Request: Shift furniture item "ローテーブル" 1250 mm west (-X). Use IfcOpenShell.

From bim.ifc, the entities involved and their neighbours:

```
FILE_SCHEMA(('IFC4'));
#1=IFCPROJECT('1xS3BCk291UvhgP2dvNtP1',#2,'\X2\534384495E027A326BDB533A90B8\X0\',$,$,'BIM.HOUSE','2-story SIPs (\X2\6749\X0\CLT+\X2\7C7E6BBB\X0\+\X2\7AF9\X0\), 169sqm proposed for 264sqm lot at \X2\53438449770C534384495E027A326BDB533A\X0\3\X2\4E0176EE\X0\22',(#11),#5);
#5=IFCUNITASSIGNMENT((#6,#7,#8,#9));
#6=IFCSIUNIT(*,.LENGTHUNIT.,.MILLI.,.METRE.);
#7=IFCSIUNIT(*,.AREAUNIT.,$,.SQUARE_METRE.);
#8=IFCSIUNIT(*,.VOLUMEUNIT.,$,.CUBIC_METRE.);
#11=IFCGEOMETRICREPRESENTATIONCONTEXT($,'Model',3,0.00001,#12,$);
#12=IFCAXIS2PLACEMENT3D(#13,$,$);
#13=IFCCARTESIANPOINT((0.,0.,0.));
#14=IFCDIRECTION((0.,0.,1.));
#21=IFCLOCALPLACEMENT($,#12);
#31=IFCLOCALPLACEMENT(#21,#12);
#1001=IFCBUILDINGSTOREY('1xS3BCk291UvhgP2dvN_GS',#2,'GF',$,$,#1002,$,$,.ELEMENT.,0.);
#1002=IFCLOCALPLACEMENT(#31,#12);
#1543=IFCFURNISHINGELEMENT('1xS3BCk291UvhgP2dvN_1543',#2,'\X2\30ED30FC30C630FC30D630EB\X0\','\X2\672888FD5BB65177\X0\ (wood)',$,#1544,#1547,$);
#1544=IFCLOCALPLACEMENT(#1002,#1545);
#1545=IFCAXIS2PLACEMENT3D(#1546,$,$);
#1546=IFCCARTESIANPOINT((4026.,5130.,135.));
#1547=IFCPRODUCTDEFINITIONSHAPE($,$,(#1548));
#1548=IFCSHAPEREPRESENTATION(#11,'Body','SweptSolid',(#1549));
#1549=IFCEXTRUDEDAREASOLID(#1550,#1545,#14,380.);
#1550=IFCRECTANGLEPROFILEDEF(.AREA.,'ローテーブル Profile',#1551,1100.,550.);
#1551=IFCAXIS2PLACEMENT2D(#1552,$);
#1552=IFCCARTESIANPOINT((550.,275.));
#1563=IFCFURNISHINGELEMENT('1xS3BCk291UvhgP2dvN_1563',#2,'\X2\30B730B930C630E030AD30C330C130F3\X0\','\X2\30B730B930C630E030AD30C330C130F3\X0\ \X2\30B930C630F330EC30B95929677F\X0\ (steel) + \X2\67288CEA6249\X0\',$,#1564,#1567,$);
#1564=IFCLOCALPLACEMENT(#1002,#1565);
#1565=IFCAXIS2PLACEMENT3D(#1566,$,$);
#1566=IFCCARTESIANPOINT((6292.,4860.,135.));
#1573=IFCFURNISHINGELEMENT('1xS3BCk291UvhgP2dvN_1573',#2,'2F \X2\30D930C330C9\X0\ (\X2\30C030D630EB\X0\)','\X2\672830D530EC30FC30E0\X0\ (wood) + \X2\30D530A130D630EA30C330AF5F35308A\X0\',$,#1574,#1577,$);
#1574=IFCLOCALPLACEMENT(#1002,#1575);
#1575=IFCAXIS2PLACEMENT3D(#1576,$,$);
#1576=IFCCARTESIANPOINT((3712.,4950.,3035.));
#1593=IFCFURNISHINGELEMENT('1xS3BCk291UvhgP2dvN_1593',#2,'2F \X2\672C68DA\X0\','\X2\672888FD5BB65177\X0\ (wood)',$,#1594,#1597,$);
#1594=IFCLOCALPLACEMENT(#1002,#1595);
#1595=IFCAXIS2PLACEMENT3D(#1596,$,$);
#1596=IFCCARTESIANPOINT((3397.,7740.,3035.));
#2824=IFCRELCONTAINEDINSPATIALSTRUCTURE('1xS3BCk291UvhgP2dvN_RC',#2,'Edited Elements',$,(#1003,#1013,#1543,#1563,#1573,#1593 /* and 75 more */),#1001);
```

```python
import ifcopenshell
import ifcopenshell.api.geometry
import ifcopenshell.util.placement
import ifcopenshell.util.unit

model = ifcopenshell.open("bim.ifc")
unit_scale = ifcopenshell.util.unit.calculate_unit_scale(model)

item = model.by_guid("1xS3BCk291UvhgP2dvN_1543")
matrix = ifcopenshell.util.placement.get_local_placement(item.ObjectPlacement)
matrix[0, 3] -= 1.25 / unit_scale
ifcopenshell.api.geometry.edit_object_placement(model, product=item, matrix=matrix, is_si=False)

print(ifcopenshell.util.placement.get_local_placement(item.ObjectPlacement).round(3) + 0.0)

model.write("bim_updated.ifc")
```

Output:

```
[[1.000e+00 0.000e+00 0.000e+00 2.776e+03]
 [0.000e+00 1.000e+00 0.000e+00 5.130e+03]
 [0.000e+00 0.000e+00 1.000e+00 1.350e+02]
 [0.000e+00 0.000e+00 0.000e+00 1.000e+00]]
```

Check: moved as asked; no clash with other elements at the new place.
